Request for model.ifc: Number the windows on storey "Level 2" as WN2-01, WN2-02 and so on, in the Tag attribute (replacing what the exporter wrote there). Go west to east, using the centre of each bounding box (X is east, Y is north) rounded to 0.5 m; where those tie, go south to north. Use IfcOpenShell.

First a look at what the model holds.

```python
import ifcopenshell
import ifcopenshell.util.element
import ifcopenshell.util.placement

model = ifcopenshell.open("model.ifc")
print(model.schema)
storey = next(s for s in model.by_type("IfcBuildingStorey") if s.Name == "Level 2")
windows = [e for e in ifcopenshell.util.element.get_decomposition(storey) if e.is_a("IfcWindow")]
for e in sorted(windows, key=lambda e: e.id()):
    origin = ifcopenshell.util.placement.get_local_placement(e.ObjectPlacement)[:3, 3]
    print(e.id(), e.Tag, e.Name, origin.round(2) + 0.0, sep=" | ")
```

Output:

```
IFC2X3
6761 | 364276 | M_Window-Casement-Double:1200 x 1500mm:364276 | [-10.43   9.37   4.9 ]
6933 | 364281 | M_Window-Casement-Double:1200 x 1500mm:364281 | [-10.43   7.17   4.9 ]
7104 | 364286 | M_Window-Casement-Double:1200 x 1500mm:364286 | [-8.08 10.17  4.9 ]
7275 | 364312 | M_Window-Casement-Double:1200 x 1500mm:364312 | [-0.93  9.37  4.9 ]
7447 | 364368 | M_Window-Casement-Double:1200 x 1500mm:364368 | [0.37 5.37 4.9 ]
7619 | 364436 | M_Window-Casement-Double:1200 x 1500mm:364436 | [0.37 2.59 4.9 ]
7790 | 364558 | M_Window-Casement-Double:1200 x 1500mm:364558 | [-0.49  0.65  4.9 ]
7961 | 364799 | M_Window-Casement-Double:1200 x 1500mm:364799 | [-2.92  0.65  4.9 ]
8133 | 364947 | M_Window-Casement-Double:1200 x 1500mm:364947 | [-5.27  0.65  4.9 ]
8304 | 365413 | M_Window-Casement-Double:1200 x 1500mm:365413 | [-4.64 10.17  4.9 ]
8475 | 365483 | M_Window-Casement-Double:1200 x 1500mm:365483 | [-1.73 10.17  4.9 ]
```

```python
import ifcopenshell
import ifcopenshell.geom
import ifcopenshell.util.element
import ifcopenshell.util.shape

model = ifcopenshell.open("model.ifc")
settings = ifcopenshell.geom.settings()
settings.set("use-world-coords", True)


def centre(element):
    shape = ifcopenshell.geom.create_shape(settings, element)
    return ifcopenshell.util.shape.get_bbox_centroid(shape.geometry)


storey = next(s for s in model.by_type("IfcBuildingStorey") if s.Name == "Level 2")
windows = [e for e in ifcopenshell.util.element.get_decomposition(storey) if e.is_a("IfcWindow")]

# Insertion points can sit at a corner or the storey origin, so sort by the geometry (in metres).
centres = {e: centre(e) for e in windows}
windows.sort(key=lambda e: (round(centres[e][0] / 0.5), centres[e][1]))

for i, e in enumerate(windows, start=1):
    number = f"WN2-{i:02d}"
    e.Tag = number
    print(e.id(), number)

model.write("model_v2.ifc")
```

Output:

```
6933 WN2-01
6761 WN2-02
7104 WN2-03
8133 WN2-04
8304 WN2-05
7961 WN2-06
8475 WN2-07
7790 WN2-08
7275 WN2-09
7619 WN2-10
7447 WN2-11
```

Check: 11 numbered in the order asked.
